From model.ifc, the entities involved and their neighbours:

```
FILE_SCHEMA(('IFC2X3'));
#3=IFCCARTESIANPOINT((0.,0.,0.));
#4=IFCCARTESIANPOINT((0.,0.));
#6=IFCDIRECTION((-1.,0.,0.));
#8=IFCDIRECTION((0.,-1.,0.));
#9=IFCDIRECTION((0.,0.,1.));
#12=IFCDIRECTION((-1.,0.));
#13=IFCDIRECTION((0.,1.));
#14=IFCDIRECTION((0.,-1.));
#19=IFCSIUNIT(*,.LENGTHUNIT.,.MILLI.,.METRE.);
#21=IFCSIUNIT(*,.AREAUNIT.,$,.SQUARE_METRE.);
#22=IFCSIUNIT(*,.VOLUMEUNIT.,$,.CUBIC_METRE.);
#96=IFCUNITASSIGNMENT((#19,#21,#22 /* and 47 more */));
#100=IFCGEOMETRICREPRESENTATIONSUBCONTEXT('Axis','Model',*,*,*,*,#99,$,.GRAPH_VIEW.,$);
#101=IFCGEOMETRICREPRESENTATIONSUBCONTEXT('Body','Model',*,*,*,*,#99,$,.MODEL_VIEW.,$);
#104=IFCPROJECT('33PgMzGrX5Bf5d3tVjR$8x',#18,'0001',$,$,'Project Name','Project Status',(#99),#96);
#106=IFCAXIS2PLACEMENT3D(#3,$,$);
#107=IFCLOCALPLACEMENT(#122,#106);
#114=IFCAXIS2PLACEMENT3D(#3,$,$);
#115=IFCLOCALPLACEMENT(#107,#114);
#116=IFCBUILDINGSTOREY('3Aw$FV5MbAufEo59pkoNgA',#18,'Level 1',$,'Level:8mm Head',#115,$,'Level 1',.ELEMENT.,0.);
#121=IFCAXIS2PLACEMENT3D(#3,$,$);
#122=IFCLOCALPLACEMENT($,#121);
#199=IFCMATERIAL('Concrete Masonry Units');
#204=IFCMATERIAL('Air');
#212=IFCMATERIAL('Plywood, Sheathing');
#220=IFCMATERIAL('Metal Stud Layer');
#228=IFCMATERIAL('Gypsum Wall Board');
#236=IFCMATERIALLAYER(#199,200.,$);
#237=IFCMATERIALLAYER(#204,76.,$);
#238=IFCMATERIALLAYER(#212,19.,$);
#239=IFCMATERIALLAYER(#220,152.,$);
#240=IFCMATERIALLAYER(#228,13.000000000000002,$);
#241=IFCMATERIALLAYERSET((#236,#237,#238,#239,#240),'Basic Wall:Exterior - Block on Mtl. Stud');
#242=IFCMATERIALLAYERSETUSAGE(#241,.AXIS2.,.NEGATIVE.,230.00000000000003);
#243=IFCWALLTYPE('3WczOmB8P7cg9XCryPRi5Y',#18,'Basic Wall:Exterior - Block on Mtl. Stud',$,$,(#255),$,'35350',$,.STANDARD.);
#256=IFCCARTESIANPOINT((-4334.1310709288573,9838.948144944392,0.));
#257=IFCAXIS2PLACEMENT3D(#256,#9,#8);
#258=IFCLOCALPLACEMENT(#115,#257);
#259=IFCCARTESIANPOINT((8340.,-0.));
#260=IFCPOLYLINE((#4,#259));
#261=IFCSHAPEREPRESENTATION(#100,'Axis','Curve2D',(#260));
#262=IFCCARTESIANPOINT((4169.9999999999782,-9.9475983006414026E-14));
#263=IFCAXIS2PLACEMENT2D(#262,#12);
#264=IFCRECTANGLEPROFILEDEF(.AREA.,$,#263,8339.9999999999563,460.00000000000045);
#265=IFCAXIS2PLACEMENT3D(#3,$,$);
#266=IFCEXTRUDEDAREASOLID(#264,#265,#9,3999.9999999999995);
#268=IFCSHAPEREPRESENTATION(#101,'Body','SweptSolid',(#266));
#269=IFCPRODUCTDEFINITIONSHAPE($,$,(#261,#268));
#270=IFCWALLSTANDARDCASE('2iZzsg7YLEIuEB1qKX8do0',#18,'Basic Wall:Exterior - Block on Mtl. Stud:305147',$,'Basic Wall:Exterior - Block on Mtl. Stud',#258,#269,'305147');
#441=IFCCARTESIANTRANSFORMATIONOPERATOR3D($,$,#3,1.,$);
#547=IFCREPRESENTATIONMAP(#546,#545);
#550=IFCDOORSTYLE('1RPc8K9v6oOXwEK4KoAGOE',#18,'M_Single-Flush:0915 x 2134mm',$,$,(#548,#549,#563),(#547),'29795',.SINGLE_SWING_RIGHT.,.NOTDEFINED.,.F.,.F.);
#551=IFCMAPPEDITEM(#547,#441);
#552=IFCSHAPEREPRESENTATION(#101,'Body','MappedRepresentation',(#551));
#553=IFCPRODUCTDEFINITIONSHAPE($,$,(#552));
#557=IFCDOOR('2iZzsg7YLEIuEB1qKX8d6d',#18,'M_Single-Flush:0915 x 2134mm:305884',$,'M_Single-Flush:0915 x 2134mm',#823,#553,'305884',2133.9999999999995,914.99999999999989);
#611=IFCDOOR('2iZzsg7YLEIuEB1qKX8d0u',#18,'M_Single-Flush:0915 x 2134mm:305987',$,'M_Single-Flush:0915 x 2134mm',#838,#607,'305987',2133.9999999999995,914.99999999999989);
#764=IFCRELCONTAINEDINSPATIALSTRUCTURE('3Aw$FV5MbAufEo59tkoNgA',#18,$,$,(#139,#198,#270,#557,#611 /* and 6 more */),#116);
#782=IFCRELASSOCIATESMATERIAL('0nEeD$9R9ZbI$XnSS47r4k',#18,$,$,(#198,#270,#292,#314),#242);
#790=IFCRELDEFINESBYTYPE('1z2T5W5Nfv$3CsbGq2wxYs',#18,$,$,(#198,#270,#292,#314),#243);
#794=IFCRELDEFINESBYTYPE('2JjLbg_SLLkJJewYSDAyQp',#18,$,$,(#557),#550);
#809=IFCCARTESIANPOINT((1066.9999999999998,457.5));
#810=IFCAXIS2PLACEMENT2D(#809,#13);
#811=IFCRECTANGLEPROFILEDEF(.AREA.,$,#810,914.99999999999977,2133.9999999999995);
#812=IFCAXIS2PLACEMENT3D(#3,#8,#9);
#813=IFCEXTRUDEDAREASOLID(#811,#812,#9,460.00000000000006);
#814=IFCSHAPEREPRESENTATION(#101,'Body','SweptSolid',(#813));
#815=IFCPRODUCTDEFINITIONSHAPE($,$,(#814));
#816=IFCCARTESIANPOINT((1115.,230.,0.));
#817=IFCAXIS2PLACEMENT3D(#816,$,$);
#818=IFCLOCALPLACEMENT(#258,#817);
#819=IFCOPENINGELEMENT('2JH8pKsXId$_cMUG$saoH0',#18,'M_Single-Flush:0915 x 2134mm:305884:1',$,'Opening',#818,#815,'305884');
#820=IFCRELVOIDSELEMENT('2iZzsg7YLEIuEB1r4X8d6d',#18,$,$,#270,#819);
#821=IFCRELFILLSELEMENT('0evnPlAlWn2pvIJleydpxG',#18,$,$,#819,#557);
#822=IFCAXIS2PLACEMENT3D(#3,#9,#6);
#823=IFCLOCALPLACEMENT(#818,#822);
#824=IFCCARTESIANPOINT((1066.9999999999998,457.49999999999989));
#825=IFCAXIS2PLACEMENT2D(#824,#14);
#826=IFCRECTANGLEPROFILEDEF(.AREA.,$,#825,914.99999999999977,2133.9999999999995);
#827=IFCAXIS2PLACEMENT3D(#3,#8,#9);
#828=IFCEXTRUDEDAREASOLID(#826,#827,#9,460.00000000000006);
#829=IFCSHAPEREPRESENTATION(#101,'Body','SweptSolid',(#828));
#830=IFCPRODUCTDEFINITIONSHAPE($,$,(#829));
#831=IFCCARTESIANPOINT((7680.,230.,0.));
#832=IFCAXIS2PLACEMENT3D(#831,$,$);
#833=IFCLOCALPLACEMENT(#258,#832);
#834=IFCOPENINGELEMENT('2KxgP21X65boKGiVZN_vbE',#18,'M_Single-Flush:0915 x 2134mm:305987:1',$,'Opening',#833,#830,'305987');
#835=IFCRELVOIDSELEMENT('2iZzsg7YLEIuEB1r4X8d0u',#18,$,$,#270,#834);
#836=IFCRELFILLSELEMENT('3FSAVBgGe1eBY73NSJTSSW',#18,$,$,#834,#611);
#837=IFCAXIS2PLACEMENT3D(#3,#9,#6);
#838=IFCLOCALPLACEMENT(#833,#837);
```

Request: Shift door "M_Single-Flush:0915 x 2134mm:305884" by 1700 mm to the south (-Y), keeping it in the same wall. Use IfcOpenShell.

```python
import ifcopenshell
import ifcopenshell.api.geometry
import ifcopenshell.util.placement
import ifcopenshell.util.unit

model = ifcopenshell.open("model.ifc")
unit_scale = ifcopenshell.util.unit.calculate_unit_scale(model)

door = model.by_guid("2iZzsg7YLEIuEB1qKX8d6d")
opening = door.FillsVoids[0].RelatingOpeningElement
wall = opening.VoidsElements[0].RelatingBuildingElement

wall_matrix = ifcopenshell.util.placement.get_local_placement(wall.ObjectPlacement)
shift = wall_matrix[:3, 0] * 1.7 / unit_scale
before = ifcopenshell.util.placement.get_local_placement(door.ObjectPlacement)[:3, 3].copy()

# The door is placed relative to its opening, so it follows when the opening moves.
matrix = ifcopenshell.util.placement.get_local_placement(opening.ObjectPlacement)
matrix[:3, 3] += shift
ifcopenshell.api.geometry.edit_object_placement(
    model, product=opening, matrix=matrix, is_si=False, should_transform_children=True
)

after = ifcopenshell.util.placement.get_local_placement(door.ObjectPlacement)[:3, 3]
print("door moved by", (after - before).round(3) + 0.0)

model.write("model_edited.ifc")
```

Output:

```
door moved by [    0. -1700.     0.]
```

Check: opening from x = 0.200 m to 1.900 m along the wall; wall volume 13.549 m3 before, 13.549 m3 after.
